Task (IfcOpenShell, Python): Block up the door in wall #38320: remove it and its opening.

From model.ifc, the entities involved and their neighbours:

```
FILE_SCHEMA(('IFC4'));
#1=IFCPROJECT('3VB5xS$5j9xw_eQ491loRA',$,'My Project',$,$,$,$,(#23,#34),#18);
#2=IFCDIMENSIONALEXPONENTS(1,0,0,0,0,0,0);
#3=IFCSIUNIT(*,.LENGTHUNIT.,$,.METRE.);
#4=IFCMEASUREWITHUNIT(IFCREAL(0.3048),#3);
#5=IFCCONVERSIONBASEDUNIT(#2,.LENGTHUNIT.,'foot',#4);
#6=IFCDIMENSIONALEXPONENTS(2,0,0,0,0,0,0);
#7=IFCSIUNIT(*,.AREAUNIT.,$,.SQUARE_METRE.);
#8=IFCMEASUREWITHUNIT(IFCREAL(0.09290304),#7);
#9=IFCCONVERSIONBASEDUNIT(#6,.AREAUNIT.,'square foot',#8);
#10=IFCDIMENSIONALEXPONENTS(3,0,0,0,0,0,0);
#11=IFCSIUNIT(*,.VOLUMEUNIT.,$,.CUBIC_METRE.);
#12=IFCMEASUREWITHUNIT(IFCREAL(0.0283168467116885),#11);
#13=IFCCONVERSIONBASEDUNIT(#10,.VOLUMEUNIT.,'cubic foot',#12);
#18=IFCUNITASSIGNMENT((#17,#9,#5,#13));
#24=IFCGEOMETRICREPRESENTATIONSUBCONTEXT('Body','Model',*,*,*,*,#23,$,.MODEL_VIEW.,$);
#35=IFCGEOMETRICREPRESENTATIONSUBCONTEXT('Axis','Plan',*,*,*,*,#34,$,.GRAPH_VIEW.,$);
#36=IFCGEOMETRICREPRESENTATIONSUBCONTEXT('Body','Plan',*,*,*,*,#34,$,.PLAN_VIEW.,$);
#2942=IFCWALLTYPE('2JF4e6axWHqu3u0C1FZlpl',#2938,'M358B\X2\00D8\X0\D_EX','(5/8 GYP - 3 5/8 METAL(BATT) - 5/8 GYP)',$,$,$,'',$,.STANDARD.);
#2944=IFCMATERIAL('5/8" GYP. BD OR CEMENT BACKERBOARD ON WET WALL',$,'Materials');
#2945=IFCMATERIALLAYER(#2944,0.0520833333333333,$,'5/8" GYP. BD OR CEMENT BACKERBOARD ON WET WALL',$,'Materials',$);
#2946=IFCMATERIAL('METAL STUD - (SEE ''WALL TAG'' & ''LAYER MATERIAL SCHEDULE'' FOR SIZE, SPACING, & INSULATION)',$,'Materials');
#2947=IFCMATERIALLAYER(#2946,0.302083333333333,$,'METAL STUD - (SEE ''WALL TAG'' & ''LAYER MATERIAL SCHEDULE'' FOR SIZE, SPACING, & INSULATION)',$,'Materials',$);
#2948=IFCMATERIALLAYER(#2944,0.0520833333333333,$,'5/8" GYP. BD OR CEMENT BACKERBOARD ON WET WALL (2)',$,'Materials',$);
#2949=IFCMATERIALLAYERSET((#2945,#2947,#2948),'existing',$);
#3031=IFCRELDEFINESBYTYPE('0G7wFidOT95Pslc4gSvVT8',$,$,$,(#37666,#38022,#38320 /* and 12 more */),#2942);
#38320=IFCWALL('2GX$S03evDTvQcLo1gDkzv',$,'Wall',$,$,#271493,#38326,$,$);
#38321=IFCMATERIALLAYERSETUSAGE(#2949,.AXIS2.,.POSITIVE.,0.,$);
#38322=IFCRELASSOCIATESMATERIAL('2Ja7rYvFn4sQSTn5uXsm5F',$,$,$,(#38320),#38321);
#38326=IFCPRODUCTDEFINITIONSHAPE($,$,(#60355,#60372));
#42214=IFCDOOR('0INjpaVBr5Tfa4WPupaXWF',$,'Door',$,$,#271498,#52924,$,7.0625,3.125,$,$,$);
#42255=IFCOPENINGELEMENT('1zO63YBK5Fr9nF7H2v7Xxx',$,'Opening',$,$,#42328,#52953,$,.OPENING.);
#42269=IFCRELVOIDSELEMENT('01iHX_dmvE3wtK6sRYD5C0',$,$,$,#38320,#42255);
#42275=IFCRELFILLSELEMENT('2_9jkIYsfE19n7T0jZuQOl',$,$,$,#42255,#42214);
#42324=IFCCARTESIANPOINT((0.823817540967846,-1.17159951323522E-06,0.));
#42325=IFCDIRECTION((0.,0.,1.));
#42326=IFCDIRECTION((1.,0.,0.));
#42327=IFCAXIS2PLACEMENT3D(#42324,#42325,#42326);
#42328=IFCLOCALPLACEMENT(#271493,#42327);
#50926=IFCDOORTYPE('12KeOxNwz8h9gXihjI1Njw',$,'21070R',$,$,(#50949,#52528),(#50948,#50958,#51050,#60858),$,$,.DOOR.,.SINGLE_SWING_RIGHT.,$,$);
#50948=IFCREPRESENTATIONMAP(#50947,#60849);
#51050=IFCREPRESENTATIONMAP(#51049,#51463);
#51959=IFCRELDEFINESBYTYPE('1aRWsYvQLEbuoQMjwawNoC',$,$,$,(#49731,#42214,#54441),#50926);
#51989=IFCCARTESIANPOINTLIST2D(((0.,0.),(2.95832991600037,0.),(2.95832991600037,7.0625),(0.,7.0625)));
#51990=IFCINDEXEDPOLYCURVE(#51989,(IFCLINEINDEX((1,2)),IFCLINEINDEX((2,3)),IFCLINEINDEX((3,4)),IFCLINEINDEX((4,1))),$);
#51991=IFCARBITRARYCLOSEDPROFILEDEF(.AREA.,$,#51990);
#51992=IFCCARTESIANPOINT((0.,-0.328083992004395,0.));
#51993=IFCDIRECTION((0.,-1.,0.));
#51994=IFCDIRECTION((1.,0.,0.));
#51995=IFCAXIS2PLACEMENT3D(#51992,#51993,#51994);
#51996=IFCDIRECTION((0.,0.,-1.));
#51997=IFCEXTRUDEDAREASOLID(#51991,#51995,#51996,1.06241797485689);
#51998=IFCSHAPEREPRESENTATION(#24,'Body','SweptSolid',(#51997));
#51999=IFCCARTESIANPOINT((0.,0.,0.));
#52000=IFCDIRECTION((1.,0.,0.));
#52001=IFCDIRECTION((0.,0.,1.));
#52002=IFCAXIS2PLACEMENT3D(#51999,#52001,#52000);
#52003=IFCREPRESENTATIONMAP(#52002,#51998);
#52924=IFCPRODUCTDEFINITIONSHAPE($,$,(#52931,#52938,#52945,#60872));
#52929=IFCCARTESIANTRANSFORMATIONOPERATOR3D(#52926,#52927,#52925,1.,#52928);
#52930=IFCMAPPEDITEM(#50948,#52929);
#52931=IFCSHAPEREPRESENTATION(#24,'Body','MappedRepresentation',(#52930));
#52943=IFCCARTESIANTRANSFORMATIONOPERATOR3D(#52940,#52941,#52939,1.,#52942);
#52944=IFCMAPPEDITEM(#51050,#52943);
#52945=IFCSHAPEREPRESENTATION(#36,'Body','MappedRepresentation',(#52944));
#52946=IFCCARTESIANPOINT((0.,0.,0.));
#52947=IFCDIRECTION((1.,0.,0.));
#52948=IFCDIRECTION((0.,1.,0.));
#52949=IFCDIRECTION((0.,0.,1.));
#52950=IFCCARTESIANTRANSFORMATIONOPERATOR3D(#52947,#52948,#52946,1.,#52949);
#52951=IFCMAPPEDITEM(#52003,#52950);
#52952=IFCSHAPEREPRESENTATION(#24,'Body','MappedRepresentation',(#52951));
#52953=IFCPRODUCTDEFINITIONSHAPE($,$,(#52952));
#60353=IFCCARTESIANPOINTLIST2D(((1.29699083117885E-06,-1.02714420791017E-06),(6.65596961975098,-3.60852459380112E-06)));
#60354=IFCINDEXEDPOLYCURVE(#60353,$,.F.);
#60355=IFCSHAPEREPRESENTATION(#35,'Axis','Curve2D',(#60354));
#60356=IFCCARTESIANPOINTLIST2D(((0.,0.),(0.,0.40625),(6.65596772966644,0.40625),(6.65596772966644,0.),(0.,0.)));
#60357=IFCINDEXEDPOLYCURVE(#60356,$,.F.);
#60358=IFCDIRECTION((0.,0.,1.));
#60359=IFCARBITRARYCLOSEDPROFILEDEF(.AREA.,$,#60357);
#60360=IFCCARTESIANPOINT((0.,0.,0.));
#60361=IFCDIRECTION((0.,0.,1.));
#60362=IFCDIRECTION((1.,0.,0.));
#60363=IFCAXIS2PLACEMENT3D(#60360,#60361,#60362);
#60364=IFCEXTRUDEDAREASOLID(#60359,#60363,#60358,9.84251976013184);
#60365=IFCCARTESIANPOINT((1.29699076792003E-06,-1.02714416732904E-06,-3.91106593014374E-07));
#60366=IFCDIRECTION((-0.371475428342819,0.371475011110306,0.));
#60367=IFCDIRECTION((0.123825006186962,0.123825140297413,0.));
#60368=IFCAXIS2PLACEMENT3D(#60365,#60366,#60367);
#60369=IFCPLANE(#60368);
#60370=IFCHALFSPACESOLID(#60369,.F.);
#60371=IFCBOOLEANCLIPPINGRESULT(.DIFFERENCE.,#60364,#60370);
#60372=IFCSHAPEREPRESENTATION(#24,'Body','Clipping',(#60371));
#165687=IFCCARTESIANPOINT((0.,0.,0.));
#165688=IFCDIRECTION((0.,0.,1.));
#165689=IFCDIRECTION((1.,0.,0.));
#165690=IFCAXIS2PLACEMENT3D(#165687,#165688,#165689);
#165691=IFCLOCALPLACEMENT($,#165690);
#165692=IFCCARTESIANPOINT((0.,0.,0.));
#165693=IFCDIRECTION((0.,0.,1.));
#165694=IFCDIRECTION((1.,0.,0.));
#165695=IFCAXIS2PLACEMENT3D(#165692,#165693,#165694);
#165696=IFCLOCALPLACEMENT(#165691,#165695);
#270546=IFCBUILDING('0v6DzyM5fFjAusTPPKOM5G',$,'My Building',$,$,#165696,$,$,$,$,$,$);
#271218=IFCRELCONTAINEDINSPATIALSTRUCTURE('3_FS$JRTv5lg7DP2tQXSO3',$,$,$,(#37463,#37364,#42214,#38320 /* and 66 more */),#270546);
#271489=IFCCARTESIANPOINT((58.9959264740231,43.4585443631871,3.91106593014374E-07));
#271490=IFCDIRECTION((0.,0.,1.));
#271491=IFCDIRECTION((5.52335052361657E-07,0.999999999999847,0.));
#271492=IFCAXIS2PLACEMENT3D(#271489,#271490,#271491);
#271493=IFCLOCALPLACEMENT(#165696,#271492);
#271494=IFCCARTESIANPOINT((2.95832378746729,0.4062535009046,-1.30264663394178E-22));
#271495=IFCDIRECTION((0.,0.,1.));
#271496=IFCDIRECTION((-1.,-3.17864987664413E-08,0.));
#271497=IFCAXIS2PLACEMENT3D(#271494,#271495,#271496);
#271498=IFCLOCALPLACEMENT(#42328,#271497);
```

```python
import ifcopenshell
import ifcopenshell.api.feature
import ifcopenshell.api.root
import ifcopenshell.geom
import ifcopenshell.util.shape

model = ifcopenshell.open("model.ifc")
settings = ifcopenshell.geom.settings()


def volume(element):
    """Net volume in cubic metres, openings subtracted."""
    shape = ifcopenshell.geom.create_shape(settings, element)
    return ifcopenshell.util.shape.get_volume(shape.geometry)


door = model.by_guid("0INjpaVBr5Tfa4WPupaXWF")
opening = door.FillsVoids[0].RelatingOpeningElement
wall = opening.VoidsElements[0].RelatingBuildingElement
before = volume(wall)

ifcopenshell.api.root.remove_product(model, product=door)
ifcopenshell.api.feature.remove_feature(model, feature=opening)

after = volume(wall)

print(f"wall volume {before:.3f} -> {after:.3f} m3")

model.write("model_edited.ifc")
```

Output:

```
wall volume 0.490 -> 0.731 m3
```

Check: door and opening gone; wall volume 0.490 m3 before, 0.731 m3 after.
